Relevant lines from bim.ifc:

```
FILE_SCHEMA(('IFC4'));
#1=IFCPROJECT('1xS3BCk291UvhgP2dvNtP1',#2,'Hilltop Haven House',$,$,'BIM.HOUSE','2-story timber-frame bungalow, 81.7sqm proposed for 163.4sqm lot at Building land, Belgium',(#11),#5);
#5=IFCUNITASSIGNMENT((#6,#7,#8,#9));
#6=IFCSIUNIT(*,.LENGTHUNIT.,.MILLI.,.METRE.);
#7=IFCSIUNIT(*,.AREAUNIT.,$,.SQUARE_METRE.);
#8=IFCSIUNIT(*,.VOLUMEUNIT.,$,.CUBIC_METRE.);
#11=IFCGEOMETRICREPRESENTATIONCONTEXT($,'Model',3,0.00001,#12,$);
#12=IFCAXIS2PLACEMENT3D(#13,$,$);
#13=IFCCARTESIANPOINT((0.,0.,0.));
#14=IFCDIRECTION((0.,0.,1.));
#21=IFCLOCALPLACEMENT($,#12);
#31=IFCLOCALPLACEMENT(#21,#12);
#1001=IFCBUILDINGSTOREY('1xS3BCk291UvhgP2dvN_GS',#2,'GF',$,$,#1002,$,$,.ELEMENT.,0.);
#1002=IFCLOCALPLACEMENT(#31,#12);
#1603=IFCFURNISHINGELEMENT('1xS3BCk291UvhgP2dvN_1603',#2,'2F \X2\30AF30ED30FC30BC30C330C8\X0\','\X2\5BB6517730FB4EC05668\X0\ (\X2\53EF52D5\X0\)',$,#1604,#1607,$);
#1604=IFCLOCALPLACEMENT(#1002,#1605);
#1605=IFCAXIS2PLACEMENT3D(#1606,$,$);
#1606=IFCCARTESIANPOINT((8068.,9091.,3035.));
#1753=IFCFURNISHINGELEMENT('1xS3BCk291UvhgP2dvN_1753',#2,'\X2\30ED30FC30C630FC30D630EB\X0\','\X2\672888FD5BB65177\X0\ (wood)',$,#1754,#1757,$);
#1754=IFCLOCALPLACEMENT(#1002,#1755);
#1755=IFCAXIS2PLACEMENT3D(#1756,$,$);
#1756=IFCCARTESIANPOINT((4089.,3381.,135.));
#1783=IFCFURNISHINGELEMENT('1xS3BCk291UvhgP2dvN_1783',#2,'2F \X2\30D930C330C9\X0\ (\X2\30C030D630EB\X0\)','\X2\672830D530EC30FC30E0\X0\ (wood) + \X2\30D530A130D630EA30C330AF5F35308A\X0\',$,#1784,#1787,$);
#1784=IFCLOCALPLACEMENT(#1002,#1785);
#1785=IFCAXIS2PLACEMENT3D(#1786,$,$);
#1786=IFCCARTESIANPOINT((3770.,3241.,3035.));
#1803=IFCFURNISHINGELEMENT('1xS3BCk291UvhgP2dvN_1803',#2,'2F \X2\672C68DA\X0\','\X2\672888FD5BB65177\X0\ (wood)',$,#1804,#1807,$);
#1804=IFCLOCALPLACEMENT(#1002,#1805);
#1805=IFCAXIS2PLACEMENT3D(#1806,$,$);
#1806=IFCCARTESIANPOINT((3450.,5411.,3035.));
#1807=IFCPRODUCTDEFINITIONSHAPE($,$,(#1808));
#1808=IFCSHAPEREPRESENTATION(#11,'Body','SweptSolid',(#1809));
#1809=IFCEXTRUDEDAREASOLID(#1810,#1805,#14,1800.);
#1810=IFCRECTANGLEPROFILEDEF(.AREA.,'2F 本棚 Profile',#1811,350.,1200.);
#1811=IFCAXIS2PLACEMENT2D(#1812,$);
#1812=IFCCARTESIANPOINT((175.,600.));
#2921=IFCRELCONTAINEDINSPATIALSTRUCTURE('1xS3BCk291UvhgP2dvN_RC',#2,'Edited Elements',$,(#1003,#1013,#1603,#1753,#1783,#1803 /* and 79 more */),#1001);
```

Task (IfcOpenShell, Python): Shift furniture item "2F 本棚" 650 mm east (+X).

```python
import ifcopenshell
import ifcopenshell.api.geometry
import ifcopenshell.util.placement
import ifcopenshell.util.unit

model = ifcopenshell.open("bim.ifc")
unit_scale = ifcopenshell.util.unit.calculate_unit_scale(model)

item = model.by_guid("1xS3BCk291UvhgP2dvN_1803")
matrix = ifcopenshell.util.placement.get_local_placement(item.ObjectPlacement)
matrix[0, 3] += 0.65 / unit_scale
ifcopenshell.api.geometry.edit_object_placement(model, product=item, matrix=matrix, is_si=False)

print(ifcopenshell.util.placement.get_local_placement(item.ObjectPlacement).round(3) + 0.0)

model.write("bim_edited.ifc")
```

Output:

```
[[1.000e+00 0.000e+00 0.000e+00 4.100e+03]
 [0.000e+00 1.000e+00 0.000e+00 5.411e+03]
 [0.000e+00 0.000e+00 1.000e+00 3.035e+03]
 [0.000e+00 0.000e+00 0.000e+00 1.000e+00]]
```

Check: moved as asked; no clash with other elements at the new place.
